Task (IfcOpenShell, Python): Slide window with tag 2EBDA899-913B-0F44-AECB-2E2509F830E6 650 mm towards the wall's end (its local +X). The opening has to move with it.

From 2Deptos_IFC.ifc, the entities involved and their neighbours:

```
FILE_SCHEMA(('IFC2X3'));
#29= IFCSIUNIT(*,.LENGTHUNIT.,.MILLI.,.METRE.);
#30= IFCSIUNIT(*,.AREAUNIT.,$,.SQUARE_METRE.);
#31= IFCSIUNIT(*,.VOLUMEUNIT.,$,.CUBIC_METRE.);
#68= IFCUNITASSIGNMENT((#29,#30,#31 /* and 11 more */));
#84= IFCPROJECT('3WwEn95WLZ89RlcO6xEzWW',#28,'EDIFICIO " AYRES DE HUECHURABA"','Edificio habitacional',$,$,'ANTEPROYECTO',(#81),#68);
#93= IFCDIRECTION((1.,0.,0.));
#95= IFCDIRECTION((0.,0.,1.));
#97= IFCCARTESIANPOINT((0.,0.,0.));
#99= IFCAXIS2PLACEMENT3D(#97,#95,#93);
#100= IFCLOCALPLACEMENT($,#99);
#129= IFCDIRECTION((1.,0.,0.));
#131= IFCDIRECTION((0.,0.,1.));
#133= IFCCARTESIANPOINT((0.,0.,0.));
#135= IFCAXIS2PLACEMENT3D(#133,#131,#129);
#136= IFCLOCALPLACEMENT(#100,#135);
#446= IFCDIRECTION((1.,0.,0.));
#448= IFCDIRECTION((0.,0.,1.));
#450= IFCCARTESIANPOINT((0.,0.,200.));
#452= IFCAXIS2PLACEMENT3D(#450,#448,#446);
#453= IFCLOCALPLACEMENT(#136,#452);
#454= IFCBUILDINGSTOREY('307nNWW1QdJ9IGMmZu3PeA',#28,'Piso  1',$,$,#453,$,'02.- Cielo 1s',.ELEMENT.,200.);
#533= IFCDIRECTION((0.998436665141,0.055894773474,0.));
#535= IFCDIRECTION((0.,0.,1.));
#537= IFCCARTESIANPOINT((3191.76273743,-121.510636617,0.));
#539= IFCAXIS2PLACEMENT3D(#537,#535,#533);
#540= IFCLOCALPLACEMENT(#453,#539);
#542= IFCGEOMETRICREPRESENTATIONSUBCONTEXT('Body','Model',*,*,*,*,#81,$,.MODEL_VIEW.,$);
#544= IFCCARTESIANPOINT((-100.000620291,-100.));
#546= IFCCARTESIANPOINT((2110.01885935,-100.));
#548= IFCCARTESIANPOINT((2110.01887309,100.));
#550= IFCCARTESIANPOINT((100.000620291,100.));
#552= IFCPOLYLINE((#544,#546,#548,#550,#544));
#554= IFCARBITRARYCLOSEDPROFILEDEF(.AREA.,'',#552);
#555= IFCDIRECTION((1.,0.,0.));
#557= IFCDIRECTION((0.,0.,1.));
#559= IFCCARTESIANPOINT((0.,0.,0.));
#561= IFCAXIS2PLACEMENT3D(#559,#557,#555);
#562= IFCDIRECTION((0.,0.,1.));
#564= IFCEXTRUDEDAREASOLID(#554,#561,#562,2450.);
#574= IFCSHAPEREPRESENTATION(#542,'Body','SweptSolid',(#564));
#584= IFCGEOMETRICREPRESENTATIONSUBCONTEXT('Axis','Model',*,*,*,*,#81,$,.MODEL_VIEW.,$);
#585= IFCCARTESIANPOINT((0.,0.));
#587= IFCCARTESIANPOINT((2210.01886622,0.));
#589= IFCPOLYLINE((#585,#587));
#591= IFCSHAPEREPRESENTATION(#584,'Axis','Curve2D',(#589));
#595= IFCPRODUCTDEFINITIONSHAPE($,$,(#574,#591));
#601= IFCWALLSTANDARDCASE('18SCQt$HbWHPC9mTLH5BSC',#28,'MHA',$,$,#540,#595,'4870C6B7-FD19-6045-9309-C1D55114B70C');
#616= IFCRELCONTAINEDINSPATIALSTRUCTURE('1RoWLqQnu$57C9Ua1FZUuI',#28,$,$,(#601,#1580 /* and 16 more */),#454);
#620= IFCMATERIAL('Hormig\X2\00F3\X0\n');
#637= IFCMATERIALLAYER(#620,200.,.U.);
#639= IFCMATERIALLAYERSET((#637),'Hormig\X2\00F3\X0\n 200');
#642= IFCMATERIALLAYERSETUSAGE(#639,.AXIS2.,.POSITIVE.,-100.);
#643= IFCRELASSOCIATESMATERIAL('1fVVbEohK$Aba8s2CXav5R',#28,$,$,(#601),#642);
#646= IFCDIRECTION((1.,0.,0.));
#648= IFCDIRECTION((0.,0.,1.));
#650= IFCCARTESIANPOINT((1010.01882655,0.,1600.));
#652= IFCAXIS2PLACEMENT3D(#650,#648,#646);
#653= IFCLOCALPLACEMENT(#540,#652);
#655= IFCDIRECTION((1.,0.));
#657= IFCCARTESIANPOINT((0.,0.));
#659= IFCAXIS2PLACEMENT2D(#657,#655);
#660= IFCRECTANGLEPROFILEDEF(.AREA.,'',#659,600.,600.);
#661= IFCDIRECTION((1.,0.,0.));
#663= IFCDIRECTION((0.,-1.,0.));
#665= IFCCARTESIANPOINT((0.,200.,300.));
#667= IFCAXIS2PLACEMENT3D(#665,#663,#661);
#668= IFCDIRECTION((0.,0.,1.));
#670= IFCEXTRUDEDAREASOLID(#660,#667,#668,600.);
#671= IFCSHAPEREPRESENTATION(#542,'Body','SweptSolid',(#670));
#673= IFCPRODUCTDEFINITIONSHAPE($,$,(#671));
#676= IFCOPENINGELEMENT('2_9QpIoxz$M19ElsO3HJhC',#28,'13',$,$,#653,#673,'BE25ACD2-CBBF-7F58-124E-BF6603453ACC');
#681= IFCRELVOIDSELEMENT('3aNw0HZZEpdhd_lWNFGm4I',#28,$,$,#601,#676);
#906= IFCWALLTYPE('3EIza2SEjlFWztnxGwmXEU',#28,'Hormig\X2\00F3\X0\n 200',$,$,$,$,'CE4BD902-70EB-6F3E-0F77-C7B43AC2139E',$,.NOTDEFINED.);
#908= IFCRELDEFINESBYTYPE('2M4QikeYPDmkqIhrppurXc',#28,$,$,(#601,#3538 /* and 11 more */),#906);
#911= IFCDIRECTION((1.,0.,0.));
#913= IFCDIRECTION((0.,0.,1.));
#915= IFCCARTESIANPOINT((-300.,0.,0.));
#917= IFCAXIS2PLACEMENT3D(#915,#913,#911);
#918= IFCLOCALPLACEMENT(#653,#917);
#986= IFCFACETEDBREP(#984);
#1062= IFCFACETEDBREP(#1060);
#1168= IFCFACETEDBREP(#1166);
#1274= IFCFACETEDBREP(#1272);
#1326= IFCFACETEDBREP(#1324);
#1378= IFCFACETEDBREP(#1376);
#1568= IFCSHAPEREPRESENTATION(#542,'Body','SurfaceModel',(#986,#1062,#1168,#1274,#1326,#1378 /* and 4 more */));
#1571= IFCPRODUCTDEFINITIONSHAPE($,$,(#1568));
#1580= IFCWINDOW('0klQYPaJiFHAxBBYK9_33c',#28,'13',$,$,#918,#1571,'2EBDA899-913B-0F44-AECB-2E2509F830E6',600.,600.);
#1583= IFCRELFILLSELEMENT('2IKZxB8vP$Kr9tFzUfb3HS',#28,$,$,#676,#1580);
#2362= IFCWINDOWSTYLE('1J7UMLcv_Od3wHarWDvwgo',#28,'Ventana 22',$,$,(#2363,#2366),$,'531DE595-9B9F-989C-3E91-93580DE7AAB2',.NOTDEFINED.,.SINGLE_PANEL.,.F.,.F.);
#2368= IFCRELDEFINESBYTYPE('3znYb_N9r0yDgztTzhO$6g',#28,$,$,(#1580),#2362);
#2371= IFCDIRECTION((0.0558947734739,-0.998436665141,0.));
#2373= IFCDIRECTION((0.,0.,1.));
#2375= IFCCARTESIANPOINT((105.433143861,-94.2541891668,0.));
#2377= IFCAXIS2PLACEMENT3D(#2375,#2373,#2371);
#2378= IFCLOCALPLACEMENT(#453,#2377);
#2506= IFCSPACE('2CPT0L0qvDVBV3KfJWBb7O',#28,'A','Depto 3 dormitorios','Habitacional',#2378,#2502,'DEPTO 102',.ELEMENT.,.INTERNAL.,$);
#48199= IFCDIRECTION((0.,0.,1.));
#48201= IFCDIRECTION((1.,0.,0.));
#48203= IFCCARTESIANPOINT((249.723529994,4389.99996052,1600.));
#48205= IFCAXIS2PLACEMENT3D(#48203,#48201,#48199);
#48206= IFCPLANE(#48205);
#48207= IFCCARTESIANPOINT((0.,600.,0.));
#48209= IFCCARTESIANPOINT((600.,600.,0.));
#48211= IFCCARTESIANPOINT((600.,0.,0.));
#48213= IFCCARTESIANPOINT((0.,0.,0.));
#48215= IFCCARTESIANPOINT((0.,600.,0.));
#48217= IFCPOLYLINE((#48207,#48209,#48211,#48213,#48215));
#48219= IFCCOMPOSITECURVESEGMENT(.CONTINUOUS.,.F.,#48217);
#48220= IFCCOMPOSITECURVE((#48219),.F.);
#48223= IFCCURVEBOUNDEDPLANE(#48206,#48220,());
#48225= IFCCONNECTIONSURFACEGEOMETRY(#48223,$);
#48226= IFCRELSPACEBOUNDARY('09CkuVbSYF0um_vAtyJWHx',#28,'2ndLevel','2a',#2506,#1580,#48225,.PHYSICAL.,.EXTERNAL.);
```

```python
import numpy as np
import ifcopenshell
import ifcopenshell.api.geometry
import ifcopenshell.util.placement
import ifcopenshell.util.unit

model = ifcopenshell.open("2Deptos_IFC.ifc")
unit_scale = ifcopenshell.util.unit.calculate_unit_scale(model)

window = model.by_guid("0klQYPaJiFHAxBBYK9_33c")
opening = window.FillsVoids[0].RelatingOpeningElement
wall = opening.VoidsElements[0].RelatingBuildingElement

wall_matrix = ifcopenshell.util.placement.get_local_placement(wall.ObjectPlacement)
shift = wall_matrix[:3, 0] * 0.65 / unit_scale
before = ifcopenshell.util.placement.get_local_placement(window.ObjectPlacement)[:3, 3].copy()

# The window is placed relative to its opening, so it follows when the opening moves.
matrix = ifcopenshell.util.placement.get_local_placement(opening.ObjectPlacement)
matrix[:3, 3] += shift
ifcopenshell.api.geometry.edit_object_placement(
    model, product=opening, matrix=matrix, is_si=False, should_transform_children=True
)

# Space boundary surfaces are stored in each space's coordinates; move them too.
for rel in window.ProvidesBoundaries:
    if not rel.ConnectionGeometry:
        continue
    surface = rel.ConnectionGeometry.SurfaceOnRelatingElement.BasisSurface
    space_matrix = ifcopenshell.util.placement.get_local_placement(rel.RelatingSpace.ObjectPlacement)
    point = np.array(surface.Position.Location.Coordinates) + space_matrix[:3, :3].T @ shift
    surface.Position = model.createIfcAxis2Placement3D(
        model.createIfcCartesianPoint(point.tolist()), surface.Position.Axis, surface.Position.RefDirection
    )

after = ifcopenshell.util.placement.get_local_placement(window.ObjectPlacement)[:3, 3]
print("window moved by", (after - before).round(3) + 0.0)

model.write("2Deptos_IFC_v2.ifc")
```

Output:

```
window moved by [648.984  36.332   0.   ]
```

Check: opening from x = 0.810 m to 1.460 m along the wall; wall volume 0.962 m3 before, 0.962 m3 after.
